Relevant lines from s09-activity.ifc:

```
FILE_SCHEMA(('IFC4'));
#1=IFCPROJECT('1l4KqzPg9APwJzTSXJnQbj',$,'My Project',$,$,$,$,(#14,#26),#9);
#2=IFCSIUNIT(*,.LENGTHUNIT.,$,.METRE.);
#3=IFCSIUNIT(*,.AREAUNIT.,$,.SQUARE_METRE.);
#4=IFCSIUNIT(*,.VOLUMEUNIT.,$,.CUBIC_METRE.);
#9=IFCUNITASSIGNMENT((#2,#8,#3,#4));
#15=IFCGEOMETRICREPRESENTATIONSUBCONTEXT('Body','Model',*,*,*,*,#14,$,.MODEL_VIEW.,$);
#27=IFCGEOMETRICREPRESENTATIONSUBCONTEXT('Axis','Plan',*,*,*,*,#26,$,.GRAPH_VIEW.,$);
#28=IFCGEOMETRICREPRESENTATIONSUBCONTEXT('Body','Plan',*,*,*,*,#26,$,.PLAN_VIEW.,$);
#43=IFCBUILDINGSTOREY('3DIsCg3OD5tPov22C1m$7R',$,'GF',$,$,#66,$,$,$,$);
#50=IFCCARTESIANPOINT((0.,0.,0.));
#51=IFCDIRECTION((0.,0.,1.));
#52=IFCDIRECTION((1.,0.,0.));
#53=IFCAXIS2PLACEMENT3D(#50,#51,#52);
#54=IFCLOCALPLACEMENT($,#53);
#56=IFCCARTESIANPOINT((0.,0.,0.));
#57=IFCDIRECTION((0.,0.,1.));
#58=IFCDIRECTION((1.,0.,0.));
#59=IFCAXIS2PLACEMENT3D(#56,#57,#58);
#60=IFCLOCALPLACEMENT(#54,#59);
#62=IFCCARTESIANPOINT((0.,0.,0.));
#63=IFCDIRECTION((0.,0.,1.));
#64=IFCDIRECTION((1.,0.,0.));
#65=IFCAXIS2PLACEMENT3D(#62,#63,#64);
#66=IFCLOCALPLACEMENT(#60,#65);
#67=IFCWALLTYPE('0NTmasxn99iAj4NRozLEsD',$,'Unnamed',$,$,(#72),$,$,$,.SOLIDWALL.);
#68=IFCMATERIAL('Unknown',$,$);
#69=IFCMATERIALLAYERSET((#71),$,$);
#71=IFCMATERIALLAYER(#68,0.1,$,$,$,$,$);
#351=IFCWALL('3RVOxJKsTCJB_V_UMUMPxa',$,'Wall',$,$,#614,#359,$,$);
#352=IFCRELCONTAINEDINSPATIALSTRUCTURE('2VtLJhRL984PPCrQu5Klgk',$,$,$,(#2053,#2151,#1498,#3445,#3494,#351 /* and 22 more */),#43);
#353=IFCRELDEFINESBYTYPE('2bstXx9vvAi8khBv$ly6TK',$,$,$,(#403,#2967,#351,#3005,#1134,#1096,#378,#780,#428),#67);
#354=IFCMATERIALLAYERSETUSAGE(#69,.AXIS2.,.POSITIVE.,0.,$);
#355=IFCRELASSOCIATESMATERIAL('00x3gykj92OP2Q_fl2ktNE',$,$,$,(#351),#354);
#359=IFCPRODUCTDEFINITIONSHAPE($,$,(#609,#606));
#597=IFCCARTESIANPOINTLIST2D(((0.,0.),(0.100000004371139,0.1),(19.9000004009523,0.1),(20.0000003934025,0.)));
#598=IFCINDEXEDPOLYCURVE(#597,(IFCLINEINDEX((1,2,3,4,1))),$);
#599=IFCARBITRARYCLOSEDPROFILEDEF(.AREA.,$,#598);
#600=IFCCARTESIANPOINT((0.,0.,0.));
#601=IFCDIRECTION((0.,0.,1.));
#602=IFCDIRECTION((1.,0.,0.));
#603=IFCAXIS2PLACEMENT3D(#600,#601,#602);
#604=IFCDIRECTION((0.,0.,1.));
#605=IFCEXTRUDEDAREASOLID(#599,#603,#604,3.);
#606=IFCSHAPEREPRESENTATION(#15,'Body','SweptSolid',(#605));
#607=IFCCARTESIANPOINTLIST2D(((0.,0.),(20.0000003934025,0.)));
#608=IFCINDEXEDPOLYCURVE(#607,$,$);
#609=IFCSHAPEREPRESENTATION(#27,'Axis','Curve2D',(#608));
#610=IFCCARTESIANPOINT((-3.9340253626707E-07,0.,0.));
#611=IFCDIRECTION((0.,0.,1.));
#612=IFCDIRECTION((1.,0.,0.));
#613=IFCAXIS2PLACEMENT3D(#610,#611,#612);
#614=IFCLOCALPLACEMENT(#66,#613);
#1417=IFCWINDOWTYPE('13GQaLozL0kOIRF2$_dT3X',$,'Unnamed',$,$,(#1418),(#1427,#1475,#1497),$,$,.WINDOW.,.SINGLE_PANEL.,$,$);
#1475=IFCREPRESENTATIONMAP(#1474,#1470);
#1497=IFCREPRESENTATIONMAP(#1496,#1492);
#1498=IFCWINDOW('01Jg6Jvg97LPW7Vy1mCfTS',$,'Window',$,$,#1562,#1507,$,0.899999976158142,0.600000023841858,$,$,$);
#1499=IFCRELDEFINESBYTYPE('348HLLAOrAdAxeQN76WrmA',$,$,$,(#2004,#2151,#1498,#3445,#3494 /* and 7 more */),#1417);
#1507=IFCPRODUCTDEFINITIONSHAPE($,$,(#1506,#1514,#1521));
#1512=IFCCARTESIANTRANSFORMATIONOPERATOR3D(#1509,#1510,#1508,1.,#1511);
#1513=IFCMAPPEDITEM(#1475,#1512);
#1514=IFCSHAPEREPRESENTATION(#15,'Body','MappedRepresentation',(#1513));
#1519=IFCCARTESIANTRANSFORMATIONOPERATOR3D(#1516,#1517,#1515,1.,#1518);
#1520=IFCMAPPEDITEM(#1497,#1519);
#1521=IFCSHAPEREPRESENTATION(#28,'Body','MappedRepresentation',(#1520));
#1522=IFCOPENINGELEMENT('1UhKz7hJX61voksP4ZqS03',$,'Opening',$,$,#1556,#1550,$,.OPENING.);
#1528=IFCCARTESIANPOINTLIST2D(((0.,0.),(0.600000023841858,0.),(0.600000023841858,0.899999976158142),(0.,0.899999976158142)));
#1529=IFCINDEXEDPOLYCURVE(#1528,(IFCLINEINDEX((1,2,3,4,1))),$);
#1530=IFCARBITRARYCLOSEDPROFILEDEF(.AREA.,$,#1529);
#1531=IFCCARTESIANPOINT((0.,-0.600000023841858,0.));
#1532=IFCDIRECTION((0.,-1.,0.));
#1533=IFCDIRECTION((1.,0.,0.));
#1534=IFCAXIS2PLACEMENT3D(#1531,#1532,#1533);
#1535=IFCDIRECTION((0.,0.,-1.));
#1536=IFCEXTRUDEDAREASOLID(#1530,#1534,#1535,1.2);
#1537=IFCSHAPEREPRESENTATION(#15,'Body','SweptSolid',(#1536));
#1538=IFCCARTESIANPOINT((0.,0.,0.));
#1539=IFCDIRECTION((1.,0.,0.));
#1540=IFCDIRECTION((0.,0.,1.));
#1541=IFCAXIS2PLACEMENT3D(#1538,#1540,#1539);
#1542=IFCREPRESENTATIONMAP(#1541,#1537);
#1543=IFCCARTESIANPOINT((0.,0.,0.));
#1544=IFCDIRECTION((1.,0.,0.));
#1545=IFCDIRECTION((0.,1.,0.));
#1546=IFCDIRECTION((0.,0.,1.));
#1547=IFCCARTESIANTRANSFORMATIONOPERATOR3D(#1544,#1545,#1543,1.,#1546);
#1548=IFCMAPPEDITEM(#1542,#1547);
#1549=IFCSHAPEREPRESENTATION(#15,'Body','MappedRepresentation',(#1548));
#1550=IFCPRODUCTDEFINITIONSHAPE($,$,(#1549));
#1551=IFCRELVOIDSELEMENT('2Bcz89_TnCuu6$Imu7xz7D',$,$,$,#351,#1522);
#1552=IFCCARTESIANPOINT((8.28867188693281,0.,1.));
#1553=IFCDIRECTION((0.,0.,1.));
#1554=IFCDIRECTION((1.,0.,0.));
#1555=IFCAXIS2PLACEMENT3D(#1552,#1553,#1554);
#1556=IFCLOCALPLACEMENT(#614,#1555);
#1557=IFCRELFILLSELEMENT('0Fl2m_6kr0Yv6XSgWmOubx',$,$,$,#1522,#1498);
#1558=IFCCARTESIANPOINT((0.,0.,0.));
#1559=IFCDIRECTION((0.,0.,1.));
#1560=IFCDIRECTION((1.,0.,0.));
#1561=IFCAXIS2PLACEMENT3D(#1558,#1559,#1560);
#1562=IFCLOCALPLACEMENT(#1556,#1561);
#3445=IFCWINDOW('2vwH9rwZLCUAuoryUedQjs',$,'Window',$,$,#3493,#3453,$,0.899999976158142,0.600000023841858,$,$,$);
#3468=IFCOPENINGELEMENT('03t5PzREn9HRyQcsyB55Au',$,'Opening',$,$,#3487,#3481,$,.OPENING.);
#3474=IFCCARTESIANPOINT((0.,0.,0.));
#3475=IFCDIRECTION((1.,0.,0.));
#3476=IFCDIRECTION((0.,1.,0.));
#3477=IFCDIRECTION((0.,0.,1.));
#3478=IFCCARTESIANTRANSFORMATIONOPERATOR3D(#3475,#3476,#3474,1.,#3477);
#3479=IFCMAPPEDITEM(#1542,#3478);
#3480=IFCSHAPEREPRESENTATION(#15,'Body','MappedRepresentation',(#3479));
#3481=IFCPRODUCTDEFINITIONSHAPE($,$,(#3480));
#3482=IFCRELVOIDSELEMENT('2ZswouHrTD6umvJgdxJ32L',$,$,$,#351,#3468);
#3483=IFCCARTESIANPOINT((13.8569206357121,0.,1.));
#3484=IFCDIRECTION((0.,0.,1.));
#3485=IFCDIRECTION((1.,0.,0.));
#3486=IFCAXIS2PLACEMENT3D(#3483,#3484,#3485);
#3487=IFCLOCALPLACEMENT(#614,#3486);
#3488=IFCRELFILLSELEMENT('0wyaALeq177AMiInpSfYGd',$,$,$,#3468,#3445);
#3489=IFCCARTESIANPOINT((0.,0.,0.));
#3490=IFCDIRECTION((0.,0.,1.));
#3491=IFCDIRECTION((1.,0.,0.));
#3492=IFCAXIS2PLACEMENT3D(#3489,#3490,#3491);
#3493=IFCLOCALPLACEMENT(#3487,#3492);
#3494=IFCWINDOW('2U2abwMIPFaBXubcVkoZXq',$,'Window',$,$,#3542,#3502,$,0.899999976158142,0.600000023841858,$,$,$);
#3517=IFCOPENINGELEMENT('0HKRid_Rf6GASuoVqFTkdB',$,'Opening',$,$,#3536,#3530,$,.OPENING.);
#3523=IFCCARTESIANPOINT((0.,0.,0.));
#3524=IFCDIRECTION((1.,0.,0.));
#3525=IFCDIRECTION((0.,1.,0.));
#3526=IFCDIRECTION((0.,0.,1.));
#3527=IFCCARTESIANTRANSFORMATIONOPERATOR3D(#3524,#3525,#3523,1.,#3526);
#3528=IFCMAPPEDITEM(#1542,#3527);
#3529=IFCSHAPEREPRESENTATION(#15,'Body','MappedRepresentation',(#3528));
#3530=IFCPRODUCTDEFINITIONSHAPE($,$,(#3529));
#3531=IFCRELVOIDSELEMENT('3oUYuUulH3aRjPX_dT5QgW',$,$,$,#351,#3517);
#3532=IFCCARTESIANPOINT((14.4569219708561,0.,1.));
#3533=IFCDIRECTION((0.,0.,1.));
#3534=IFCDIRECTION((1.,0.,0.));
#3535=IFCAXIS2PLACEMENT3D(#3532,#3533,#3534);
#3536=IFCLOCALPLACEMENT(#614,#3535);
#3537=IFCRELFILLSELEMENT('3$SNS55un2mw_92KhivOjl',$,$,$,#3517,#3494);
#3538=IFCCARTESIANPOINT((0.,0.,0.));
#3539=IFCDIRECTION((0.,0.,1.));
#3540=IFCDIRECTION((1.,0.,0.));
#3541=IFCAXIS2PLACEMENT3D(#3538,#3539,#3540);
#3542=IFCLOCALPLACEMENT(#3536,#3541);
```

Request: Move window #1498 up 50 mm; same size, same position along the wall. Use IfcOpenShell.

```python
import numpy as np
import ifcopenshell
import ifcopenshell.api.geometry
import ifcopenshell.util.placement
import ifcopenshell.util.unit

model = ifcopenshell.open("s09-activity.ifc")
unit_scale = ifcopenshell.util.unit.calculate_unit_scale(model)

window = model.by_guid("01Jg6Jvg97LPW7Vy1mCfTS")
opening = window.FillsVoids[0].RelatingOpeningElement
dz = 0.05

shift = np.array([0.0, 0.0, dz])
# The window is placed relative to its opening, so it follows when the opening moves.
matrix = ifcopenshell.util.placement.get_local_placement(opening.ObjectPlacement)
matrix[:3, 3] += shift
ifcopenshell.api.geometry.edit_object_placement(
    model, product=opening, matrix=matrix, is_si=False, should_transform_children=True
)

print(f"moved by {dz * unit_scale:+.3f} m")

model.write("s09-activity-out.ifc")
```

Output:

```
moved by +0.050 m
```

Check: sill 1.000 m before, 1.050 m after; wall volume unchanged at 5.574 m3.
